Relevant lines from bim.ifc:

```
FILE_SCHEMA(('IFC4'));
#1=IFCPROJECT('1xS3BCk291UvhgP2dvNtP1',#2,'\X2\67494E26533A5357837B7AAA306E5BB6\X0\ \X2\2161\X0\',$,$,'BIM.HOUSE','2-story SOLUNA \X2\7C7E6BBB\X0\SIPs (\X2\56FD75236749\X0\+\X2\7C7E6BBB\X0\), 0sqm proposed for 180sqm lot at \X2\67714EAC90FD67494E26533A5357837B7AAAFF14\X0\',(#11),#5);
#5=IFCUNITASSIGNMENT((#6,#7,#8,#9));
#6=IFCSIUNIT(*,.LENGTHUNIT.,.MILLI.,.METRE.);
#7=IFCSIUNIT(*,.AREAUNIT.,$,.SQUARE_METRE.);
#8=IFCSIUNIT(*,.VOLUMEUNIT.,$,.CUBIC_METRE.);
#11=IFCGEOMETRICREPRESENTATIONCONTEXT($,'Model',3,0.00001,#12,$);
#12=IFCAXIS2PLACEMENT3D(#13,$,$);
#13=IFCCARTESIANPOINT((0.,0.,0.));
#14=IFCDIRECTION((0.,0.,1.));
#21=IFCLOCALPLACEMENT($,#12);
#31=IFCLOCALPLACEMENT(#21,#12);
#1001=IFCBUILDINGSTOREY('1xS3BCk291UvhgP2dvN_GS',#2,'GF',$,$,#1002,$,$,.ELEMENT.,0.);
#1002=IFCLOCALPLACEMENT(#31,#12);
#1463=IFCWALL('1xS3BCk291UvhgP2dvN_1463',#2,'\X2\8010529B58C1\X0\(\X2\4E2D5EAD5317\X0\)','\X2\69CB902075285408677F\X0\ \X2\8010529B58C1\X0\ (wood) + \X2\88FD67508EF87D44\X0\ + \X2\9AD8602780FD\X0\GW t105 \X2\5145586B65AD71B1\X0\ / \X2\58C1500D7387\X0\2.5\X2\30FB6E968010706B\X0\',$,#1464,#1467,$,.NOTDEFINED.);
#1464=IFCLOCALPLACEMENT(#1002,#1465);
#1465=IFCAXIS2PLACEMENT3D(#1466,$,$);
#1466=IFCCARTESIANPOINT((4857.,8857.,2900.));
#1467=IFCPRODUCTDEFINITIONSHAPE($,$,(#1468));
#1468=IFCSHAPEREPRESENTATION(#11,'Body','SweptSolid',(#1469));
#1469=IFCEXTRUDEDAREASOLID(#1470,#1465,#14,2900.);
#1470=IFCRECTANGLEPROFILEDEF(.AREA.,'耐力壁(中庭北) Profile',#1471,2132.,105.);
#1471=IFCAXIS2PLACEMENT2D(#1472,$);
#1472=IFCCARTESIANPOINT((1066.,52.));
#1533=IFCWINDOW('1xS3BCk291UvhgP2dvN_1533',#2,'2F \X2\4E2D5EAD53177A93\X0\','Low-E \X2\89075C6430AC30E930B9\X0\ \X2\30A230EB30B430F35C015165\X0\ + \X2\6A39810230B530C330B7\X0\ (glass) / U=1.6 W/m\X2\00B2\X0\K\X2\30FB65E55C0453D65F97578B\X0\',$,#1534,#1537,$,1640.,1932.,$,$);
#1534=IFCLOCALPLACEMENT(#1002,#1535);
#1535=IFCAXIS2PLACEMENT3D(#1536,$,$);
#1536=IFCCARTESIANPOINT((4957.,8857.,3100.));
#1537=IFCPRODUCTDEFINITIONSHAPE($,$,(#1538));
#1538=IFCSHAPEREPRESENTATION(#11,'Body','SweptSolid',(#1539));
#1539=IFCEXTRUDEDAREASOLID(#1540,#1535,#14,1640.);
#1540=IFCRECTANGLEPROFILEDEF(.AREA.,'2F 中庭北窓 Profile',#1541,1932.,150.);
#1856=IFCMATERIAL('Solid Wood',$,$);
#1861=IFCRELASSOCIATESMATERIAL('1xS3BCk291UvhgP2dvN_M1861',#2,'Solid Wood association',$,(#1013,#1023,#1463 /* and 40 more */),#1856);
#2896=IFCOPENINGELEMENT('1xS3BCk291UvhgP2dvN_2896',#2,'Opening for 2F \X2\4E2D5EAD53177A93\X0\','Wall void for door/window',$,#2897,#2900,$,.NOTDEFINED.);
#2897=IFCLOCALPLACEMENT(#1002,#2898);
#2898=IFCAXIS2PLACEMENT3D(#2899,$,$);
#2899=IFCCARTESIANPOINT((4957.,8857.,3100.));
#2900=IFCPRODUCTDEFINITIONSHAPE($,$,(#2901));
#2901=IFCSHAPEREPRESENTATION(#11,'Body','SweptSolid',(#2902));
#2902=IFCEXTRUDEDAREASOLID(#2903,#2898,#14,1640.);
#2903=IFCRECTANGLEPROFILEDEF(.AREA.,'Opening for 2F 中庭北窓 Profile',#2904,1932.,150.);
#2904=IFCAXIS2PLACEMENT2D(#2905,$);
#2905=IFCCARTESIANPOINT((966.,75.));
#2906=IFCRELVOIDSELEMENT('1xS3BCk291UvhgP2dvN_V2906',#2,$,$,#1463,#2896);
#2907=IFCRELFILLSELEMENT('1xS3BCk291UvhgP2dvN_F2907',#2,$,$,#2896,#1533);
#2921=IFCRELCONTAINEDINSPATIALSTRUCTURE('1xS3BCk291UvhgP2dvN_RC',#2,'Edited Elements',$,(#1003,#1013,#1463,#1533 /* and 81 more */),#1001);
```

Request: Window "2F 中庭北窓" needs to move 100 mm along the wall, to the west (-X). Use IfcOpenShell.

```python
import ifcopenshell
import ifcopenshell.api.geometry
import ifcopenshell.util.placement
import ifcopenshell.util.unit

model = ifcopenshell.open("bim.ifc")
unit_scale = ifcopenshell.util.unit.calculate_unit_scale(model)

window = model.by_id(1533)
opening = window.FillsVoids[0].RelatingOpeningElement
wall = opening.VoidsElements[0].RelatingBuildingElement

wall_matrix = ifcopenshell.util.placement.get_local_placement(wall.ObjectPlacement)
shift = wall_matrix[:3, 0] * -0.1 / unit_scale
before = ifcopenshell.util.placement.get_local_placement(window.ObjectPlacement)[:3, 3].copy()

# The window is not placed relative to its opening, so move both.
for product in (opening, window):
    matrix = ifcopenshell.util.placement.get_local_placement(product.ObjectPlacement)
    matrix[:3, 3] += shift
    ifcopenshell.api.geometry.edit_object_placement(model, product=product, matrix=matrix, is_si=False)

after = ifcopenshell.util.placement.get_local_placement(window.ObjectPlacement)[:3, 3]
print("window moved by", (after - before).round(3) + 0.0)

model.write("bim-out.ifc")
```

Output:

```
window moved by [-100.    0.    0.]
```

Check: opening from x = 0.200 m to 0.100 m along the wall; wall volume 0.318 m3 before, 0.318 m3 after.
